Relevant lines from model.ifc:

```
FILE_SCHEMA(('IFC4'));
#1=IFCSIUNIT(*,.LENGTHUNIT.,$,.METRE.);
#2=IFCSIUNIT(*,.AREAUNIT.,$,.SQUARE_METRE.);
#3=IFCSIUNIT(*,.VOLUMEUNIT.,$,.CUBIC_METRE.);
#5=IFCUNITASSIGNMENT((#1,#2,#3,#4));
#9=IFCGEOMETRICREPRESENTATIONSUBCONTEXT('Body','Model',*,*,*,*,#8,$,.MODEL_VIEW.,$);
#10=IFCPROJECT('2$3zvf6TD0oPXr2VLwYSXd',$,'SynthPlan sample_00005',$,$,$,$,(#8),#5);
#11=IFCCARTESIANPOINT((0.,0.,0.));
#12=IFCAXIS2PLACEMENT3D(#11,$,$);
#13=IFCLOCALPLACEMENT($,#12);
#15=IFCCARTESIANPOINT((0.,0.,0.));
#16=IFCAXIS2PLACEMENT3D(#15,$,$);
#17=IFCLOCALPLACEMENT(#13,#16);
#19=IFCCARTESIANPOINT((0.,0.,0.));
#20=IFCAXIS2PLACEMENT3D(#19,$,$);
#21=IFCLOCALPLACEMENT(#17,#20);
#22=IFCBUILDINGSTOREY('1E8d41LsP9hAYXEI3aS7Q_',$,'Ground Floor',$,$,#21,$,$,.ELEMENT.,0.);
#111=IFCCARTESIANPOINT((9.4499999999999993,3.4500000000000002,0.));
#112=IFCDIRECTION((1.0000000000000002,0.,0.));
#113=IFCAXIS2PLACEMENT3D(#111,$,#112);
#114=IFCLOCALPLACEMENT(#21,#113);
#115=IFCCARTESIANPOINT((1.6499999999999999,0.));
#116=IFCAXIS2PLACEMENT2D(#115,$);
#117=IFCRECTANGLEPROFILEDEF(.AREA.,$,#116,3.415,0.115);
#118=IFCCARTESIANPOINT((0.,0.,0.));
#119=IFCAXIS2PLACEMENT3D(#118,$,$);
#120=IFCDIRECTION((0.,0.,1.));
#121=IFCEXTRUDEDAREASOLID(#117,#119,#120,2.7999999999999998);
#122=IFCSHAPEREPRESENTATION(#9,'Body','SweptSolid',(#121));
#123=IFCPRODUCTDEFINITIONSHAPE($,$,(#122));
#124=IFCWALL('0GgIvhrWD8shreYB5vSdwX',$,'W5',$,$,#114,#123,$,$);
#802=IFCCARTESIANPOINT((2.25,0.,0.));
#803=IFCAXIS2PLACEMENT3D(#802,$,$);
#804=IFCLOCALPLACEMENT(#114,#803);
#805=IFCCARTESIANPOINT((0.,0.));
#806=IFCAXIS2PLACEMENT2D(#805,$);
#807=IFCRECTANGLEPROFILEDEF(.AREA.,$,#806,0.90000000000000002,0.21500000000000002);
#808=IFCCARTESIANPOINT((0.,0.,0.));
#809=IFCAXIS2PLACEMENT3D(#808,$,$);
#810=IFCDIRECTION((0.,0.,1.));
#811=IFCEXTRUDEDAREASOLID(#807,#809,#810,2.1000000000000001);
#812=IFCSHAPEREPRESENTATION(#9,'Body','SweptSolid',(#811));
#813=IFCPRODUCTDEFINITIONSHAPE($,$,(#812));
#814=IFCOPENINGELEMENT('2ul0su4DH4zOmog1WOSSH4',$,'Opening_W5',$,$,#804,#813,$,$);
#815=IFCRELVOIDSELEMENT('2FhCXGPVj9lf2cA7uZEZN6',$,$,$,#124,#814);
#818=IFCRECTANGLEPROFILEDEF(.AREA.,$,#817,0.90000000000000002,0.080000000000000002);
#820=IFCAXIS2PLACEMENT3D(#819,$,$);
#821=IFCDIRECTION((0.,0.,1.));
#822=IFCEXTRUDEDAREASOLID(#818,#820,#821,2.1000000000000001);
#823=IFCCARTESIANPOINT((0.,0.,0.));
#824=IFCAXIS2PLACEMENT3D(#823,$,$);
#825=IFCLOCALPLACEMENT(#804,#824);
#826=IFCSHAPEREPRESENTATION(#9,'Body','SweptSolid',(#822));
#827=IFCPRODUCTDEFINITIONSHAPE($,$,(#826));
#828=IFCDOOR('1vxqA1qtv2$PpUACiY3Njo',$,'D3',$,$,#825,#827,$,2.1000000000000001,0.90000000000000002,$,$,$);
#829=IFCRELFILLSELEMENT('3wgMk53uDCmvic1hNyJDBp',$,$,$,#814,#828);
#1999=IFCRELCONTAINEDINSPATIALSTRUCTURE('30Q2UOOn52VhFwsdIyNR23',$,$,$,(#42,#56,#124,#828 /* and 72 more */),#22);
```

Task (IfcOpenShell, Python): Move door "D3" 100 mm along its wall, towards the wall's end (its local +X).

```python
import ifcopenshell
import ifcopenshell.api.geometry
import ifcopenshell.util.placement
import ifcopenshell.util.unit

model = ifcopenshell.open("model.ifc")
unit_scale = ifcopenshell.util.unit.calculate_unit_scale(model)

door = model.by_guid("1vxqA1qtv2$PpUACiY3Njo")
opening = door.FillsVoids[0].RelatingOpeningElement
wall = opening.VoidsElements[0].RelatingBuildingElement

wall_matrix = ifcopenshell.util.placement.get_local_placement(wall.ObjectPlacement)
shift = wall_matrix[:3, 0] * 0.1 / unit_scale
before = ifcopenshell.util.placement.get_local_placement(door.ObjectPlacement)[:3, 3].copy()

# The door is placed relative to its opening, so it follows when the opening moves.
matrix = ifcopenshell.util.placement.get_local_placement(opening.ObjectPlacement)
matrix[:3, 3] += shift
ifcopenshell.api.geometry.edit_object_placement(
    model, product=opening, matrix=matrix, is_si=False, should_transform_children=True
)

after = ifcopenshell.util.placement.get_local_placement(door.ObjectPlacement)[:3, 3]
print("door moved by", (after - before).round(3) + 0.0)

model.write("model-out.ifc")
```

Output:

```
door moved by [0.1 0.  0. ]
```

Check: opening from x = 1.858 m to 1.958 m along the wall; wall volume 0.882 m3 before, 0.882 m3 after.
